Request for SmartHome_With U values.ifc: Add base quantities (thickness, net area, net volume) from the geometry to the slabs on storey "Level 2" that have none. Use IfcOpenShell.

First a look at what the model holds.

```python
import ifcopenshell
import ifcopenshell.util.element
import ifcopenshell.util.unit

model = ifcopenshell.open("SmartHome_With U values.ifc")
print(model.schema)
for unit_type in ("LENGTHUNIT", "AREAUNIT", "VOLUMEUNIT"):
    print(unit_type, ifcopenshell.util.unit.calculate_unit_scale(model, unit_type))
storey = next(s for s in model.by_type("IfcBuildingStorey") if s.Name == "Level 2")
slabs = [e for e in ifcopenshell.util.element.get_decomposition(storey) if e.is_a("IfcSlab")]
for e in sorted(slabs, key=lambda e: e.id()):
    print(e.id(), e.is_a(), e.Name, list(ifcopenshell.util.element.get_psets(e, qtos_only=True)), sep=" | ")
```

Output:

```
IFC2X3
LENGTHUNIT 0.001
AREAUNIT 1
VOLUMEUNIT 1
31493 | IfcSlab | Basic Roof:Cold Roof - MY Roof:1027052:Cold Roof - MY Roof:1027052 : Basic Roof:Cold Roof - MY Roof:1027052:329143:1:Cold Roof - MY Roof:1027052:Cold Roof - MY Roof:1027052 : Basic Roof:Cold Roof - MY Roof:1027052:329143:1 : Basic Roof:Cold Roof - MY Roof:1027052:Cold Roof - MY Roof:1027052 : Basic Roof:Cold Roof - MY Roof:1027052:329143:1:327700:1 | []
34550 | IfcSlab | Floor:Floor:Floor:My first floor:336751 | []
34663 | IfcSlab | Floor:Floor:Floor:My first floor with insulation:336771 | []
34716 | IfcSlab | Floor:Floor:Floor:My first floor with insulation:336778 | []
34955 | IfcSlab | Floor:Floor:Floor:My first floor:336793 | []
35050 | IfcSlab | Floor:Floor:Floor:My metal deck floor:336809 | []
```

```python
import ifcopenshell
import ifcopenshell.api.pset
import ifcopenshell.geom
import ifcopenshell.util.element
import ifcopenshell.util.shape
import ifcopenshell.util.unit

model = ifcopenshell.open("SmartHome_With U values.ifc")
unit_scale = ifcopenshell.util.unit.calculate_unit_scale(model)
area_scale = ifcopenshell.util.unit.calculate_unit_scale(model, "AREAUNIT")
volume_scale = ifcopenshell.util.unit.calculate_unit_scale(model, "VOLUMEUNIT")
settings = ifcopenshell.geom.settings()

storey = next(s for s in model.by_type("IfcBuildingStorey") if s.Name == "Level 2")
slabs = [e for e in ifcopenshell.util.element.get_decomposition(storey) if e.is_a("IfcSlab")]

for e in sorted(slabs, key=lambda e: e.id()):
    if ifcopenshell.util.element.get_psets(e, qtos_only=True, should_inherit=False):
        continue
    # Geometry comes back in metres, in the element's own axes.
    shape = ifcopenshell.geom.create_shape(settings, e)
    values = {
        "Width": ifcopenshell.util.shape.get_z(shape.geometry) / unit_scale,
        "NetArea": ifcopenshell.util.shape.get_footprint_area(shape.geometry) / area_scale,
        "NetVolume": ifcopenshell.util.shape.get_volume(shape.geometry) / volume_scale,
    }
    qto = ifcopenshell.api.pset.add_qto(model, product=e, name="BaseQuantities")
    ifcopenshell.api.pset.edit_qto(model, qto=qto, properties=values)
    print(e.id(), {k: round(v, 3) for k, v in values.items()})

model.write("SmartHome_With U values-out.ifc")
```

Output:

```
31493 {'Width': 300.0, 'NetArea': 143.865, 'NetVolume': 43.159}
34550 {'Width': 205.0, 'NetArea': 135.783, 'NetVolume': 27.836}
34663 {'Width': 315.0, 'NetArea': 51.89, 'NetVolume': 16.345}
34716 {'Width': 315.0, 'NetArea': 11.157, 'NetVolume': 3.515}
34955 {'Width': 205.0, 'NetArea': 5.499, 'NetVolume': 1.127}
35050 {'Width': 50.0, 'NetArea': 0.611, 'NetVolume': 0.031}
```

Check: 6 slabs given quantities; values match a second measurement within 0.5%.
